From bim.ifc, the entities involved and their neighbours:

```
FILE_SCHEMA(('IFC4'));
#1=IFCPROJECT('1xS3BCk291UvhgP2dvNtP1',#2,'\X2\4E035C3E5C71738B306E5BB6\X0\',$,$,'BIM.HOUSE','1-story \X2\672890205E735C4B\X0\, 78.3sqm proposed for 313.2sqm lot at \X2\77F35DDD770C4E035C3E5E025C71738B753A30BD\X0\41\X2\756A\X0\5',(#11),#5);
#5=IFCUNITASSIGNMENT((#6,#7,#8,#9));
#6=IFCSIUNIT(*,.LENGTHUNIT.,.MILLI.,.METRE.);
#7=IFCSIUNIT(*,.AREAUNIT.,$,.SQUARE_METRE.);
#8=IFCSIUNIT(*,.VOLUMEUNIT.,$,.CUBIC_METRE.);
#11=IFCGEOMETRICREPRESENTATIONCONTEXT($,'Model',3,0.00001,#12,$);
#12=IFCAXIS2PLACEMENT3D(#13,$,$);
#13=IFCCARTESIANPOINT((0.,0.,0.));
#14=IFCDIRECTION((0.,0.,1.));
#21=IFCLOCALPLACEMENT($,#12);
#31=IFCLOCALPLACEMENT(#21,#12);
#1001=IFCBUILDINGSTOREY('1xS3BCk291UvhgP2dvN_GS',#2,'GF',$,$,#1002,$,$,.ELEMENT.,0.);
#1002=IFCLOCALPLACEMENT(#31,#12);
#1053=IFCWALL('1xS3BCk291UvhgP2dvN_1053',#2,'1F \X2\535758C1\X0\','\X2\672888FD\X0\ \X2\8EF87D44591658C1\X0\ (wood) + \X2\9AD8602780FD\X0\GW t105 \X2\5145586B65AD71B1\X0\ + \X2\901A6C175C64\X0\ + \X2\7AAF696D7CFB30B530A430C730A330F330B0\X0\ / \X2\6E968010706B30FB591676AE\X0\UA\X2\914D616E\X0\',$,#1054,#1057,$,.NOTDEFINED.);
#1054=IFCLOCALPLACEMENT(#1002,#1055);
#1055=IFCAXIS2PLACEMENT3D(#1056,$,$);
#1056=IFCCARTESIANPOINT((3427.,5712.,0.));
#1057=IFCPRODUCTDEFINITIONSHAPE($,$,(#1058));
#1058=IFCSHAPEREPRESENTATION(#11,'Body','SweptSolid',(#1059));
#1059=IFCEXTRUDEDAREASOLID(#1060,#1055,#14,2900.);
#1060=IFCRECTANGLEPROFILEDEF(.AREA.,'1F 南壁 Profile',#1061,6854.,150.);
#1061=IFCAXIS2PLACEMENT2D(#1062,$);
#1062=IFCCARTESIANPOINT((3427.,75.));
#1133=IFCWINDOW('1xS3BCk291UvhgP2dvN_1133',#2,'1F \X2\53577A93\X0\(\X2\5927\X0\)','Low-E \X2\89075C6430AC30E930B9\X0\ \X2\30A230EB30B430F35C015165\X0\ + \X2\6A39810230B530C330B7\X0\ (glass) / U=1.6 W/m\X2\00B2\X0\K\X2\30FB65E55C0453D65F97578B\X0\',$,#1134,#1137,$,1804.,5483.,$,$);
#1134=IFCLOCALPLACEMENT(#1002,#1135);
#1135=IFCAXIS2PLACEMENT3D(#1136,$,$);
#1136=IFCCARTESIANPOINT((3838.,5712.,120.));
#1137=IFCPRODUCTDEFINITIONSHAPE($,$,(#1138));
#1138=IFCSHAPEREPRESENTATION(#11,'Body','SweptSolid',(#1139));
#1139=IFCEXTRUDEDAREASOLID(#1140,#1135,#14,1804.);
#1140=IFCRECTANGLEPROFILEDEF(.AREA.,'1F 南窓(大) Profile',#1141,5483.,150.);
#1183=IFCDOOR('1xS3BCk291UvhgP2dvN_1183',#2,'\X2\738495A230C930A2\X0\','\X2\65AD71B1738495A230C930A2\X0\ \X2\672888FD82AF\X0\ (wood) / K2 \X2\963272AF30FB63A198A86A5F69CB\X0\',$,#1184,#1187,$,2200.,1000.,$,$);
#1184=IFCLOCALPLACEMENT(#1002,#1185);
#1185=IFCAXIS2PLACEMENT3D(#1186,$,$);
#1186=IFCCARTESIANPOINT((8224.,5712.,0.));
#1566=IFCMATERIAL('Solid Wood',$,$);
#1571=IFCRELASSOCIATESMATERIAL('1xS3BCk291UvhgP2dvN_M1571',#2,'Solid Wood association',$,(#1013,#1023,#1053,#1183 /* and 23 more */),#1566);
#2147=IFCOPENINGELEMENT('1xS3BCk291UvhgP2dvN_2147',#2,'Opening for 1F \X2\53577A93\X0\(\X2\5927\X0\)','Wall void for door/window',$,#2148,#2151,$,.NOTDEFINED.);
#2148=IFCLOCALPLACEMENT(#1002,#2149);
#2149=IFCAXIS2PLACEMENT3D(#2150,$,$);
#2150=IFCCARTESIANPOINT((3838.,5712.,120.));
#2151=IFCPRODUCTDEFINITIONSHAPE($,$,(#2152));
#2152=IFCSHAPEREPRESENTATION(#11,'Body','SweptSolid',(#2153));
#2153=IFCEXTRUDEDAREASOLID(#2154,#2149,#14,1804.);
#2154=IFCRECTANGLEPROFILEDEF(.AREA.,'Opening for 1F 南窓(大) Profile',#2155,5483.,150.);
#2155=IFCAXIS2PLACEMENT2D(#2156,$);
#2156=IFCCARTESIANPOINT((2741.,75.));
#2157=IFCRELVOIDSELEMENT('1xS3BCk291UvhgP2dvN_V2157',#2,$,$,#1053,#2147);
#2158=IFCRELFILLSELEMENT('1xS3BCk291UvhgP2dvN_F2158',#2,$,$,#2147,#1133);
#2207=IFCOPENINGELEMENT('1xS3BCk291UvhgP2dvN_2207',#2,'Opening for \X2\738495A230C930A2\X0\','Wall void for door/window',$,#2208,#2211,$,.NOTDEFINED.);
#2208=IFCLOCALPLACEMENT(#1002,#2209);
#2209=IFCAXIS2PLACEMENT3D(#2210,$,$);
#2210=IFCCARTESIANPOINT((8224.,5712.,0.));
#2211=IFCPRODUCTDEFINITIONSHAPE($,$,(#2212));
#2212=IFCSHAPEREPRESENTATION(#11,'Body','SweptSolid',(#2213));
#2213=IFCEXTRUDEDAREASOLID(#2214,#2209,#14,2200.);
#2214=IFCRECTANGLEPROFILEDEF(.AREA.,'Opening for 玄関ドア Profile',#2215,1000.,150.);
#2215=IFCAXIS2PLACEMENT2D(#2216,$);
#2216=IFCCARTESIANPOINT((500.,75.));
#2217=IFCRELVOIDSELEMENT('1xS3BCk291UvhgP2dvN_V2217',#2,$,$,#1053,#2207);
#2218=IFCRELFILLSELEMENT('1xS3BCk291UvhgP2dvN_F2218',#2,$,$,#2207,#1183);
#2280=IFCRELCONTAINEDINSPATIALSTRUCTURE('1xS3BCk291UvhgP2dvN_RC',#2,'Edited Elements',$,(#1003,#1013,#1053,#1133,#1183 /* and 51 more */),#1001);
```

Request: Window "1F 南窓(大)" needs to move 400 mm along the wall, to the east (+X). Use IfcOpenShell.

```python
import ifcopenshell
import ifcopenshell.api.geometry
import ifcopenshell.util.placement
import ifcopenshell.util.unit

model = ifcopenshell.open("bim.ifc")
unit_scale = ifcopenshell.util.unit.calculate_unit_scale(model)

window = model.by_guid("1xS3BCk291UvhgP2dvN_1133")
opening = window.FillsVoids[0].RelatingOpeningElement
wall = opening.VoidsElements[0].RelatingBuildingElement

wall_matrix = ifcopenshell.util.placement.get_local_placement(wall.ObjectPlacement)
shift = wall_matrix[:3, 0] * 0.4 / unit_scale
before = ifcopenshell.util.placement.get_local_placement(window.ObjectPlacement)[:3, 3].copy()

# The window is not placed relative to its opening, so move both.
for product in (opening, window):
    matrix = ifcopenshell.util.placement.get_local_placement(product.ObjectPlacement)
    matrix[:3, 3] += shift
    ifcopenshell.api.geometry.edit_object_placement(model, product=product, matrix=matrix, is_si=False)

after = ifcopenshell.util.placement.get_local_placement(window.ObjectPlacement)[:3, 3]
print("window moved by", (after - before).round(3) + 0.0)

model.write("bim_edited.ifc")
```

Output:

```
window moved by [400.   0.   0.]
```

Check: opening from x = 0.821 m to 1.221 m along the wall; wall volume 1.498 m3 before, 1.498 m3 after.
